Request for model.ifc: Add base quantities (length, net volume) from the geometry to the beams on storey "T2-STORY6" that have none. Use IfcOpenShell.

First a look at what the model holds.

```python
import ifcopenshell
import ifcopenshell.util.element
import ifcopenshell.util.unit

model = ifcopenshell.open("model.ifc")
print(model.schema)
for unit_type in ("LENGTHUNIT", "AREAUNIT", "VOLUMEUNIT"):
    print(unit_type, ifcopenshell.util.unit.calculate_unit_scale(model, unit_type))
storey = next(s for s in model.by_type("IfcBuildingStorey") if s.Name == "T2-STORY6")
beams = [e for e in ifcopenshell.util.element.get_decomposition(storey) if e.is_a("IfcBeam")]
for e in sorted(beams, key=lambda e: e.id()):
    print(e.id(), e.is_a(), e.Name, list(ifcopenshell.util.element.get_psets(e, qtos_only=True)), sep=" | ")
```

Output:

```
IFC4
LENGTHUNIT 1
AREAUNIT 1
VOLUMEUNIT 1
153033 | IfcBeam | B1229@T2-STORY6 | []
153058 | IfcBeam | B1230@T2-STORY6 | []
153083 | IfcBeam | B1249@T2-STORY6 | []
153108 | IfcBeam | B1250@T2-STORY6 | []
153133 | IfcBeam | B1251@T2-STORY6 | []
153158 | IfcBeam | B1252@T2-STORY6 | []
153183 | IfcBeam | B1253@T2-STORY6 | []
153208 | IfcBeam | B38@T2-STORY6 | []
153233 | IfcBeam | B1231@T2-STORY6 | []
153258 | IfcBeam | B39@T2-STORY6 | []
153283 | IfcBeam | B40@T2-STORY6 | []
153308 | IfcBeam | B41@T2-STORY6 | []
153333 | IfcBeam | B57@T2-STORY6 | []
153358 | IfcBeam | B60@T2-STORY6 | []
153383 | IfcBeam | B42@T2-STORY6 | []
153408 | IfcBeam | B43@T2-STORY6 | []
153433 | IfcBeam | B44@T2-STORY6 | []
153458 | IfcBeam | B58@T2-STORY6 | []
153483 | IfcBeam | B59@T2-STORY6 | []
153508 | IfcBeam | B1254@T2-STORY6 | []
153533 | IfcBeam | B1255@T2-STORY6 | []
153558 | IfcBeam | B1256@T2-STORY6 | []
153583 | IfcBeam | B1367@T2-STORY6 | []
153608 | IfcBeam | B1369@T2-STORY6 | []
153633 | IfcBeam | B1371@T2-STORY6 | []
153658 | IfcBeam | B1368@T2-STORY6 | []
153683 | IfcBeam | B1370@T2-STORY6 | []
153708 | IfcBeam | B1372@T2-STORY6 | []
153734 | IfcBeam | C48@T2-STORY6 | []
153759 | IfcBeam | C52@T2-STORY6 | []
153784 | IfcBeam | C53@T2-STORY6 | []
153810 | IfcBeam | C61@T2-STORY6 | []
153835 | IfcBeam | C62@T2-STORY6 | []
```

```python
import ifcopenshell
import ifcopenshell.api.pset
import ifcopenshell.geom
import ifcopenshell.util.element
import ifcopenshell.util.shape
import ifcopenshell.util.unit

model = ifcopenshell.open("model.ifc")
unit_scale = ifcopenshell.util.unit.calculate_unit_scale(model)
volume_scale = ifcopenshell.util.unit.calculate_unit_scale(model, "VOLUMEUNIT")
settings = ifcopenshell.geom.settings()

storey = next(s for s in model.by_type("IfcBuildingStorey") if s.Name == "T2-STORY6")
beams = [e for e in ifcopenshell.util.element.get_decomposition(storey) if e.is_a("IfcBeam")]

for e in sorted(beams, key=lambda e: e.id()):
    if ifcopenshell.util.element.get_psets(e, qtos_only=True, should_inherit=False):
        continue
    # Geometry comes back in metres, in the element's own axes.
    shape = ifcopenshell.geom.create_shape(settings, e)
    values = {
        "Length": ifcopenshell.util.shape.get_max_xyz(shape.geometry) / unit_scale,
        "NetVolume": ifcopenshell.util.shape.get_volume(shape.geometry) / volume_scale,
    }
    qto = ifcopenshell.api.pset.add_qto(model, product=e, name="Qto_BeamBaseQuantities")
    ifcopenshell.api.pset.edit_qto(model, qto=qto, properties=values)
    print(e.id(), {k: round(v, 3) for k, v in values.items()})

model.write("model_rev.ifc")
```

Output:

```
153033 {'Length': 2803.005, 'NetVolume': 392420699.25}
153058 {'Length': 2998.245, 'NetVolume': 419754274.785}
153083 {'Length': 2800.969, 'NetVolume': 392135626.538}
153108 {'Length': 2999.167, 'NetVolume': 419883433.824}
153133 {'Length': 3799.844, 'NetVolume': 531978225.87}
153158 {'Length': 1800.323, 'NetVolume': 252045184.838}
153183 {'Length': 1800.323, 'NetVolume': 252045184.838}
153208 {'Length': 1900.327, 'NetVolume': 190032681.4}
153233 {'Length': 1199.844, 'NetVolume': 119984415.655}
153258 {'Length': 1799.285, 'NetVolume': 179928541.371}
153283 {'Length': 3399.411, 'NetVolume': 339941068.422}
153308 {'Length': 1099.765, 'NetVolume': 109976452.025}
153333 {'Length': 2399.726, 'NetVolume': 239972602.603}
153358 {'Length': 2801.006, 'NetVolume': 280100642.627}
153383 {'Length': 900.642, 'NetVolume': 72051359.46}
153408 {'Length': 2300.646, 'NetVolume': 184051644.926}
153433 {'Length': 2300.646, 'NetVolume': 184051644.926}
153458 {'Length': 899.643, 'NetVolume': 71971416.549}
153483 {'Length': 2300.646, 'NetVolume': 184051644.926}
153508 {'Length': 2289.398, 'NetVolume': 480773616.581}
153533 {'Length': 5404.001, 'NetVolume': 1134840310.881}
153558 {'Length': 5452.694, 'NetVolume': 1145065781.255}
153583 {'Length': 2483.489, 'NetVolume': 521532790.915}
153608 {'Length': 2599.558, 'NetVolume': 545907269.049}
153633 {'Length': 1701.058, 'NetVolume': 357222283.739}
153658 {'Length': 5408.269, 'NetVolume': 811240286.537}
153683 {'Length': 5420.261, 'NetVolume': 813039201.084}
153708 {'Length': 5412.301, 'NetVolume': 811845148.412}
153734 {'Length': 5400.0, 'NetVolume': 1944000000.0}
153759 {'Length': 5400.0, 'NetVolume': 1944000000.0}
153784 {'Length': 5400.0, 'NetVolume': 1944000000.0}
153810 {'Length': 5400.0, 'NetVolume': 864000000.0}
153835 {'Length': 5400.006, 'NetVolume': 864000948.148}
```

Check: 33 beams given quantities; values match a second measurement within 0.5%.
